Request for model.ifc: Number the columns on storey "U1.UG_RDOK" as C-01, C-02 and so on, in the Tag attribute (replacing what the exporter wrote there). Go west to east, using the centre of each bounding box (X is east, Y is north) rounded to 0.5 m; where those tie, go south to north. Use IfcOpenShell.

First a look at what the model holds.

```python
import ifcopenshell
import ifcopenshell.util.element
import ifcopenshell.util.placement

model = ifcopenshell.open("model.ifc")
print(model.schema)
storey = next(s for s in model.by_type("IfcBuildingStorey") if s.Name == "U1.UG_RDOK")
columns = [e for e in ifcopenshell.util.element.get_decomposition(storey) if e.is_a("IfcColumn")]
for e in sorted(columns, key=lambda e: e.id()):
    origin = ifcopenshell.util.placement.get_local_placement(e.ObjectPlacement)[:3, 3]
    print(e.id(), e.Tag, e.Name, origin.round(2) + 0.0, sep=" | ")
```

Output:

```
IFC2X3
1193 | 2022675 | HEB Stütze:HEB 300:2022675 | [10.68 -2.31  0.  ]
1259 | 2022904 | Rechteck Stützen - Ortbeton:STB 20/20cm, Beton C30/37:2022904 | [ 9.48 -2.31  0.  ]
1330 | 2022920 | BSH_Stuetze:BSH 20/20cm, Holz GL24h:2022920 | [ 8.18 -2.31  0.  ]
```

```python
import ifcopenshell
import ifcopenshell.geom
import ifcopenshell.util.element
import ifcopenshell.util.shape

model = ifcopenshell.open("model.ifc")
settings = ifcopenshell.geom.settings()
settings.set("use-world-coords", True)


def centre(element):
    shape = ifcopenshell.geom.create_shape(settings, element)
    return ifcopenshell.util.shape.get_bbox_centroid(shape.geometry)


storey = next(s for s in model.by_type("IfcBuildingStorey") if s.Name == "U1.UG_RDOK")
columns = [e for e in ifcopenshell.util.element.get_decomposition(storey) if e.is_a("IfcColumn")]

# Insertion points can sit at a corner or the storey origin, so sort by the geometry (in metres).
centres = {e: centre(e) for e in columns}
columns.sort(key=lambda e: (round(centres[e][0] / 0.5), centres[e][1]))

for i, e in enumerate(columns, start=1):
    number = f"C-{i:02d}"
    e.Tag = number
    print(e.id(), number)

model.write("model_v2.ifc")
```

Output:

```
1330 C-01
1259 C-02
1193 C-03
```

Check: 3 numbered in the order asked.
